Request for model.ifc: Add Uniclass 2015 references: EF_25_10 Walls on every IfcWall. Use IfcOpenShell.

First a look at what the model holds.

```python
import ifcopenshell

model = ifcopenshell.open("model.ifc")
print(model.schema)
print("classifications:", [c.Name for c in model.by_type("IfcClassification")])
for ifc_class in ("IfcDoor", "IfcRoof", "IfcStair", "IfcWall", "IfcWindow"):
    print(ifc_class, len(model.by_type(ifc_class)))
```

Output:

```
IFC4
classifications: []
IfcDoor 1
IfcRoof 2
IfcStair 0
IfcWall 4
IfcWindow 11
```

```python
import ifcopenshell
import ifcopenshell.api.classification

model = ifcopenshell.open("model.ifc")

system = ifcopenshell.api.classification.add_classification(model, classification="Uniclass 2015")

codes = {
    "IfcWall": ("EF_25_10", "Walls"),
}
for ifc_class, (code, name) in codes.items():
    products = model.by_type(ifc_class)
    ifcopenshell.api.classification.add_reference(
        model, products=products, classification=system, identification=code, name=name
    )
    print(code, len(products))

model.write("model-out.ifc")
```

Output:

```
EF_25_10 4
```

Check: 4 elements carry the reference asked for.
